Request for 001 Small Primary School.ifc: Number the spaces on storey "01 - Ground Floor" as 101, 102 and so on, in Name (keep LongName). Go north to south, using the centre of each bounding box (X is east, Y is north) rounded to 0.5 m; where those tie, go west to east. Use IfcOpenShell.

First a look at what the model holds.

```python
import ifcopenshell
import ifcopenshell.util.element
import ifcopenshell.util.placement

model = ifcopenshell.open("001 Small Primary School.ifc")
print(model.schema)
storey = next(s for s in model.by_type("IfcBuildingStorey") if s.Name == "01 - Ground Floor")
spaces = [e for e in ifcopenshell.util.element.get_decomposition(storey) if e.is_a("IfcSpace")]
for e in sorted(spaces, key=lambda e: e.id()):
    origin = ifcopenshell.util.placement.get_local_placement(e.ObjectPlacement)[:3, 3]
    print(e.id(), e.Name, e.LongName, origin.round(2) + 0.0, sep=" | ")
```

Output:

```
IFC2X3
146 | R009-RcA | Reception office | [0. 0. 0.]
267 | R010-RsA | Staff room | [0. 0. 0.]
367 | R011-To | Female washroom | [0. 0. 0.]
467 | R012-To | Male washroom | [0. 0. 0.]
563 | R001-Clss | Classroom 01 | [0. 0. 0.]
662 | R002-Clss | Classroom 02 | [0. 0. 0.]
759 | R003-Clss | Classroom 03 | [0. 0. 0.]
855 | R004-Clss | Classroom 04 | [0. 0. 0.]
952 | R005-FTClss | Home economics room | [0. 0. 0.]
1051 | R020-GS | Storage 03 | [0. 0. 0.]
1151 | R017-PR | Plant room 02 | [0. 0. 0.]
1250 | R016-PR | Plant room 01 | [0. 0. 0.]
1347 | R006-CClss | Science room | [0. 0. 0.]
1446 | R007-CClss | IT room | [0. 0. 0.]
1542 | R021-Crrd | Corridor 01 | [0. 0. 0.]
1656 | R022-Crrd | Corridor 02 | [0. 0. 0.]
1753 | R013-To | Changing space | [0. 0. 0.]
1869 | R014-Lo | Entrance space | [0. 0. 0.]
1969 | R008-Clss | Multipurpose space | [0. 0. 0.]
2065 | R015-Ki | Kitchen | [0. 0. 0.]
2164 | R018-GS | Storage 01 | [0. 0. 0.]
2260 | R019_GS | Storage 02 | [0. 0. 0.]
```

```python
import ifcopenshell
import ifcopenshell.geom
import ifcopenshell.util.element
import ifcopenshell.util.shape

model = ifcopenshell.open("001 Small Primary School.ifc")
settings = ifcopenshell.geom.settings()
settings.set("use-world-coords", True)


def centre(element):
    shape = ifcopenshell.geom.create_shape(settings, element)
    return ifcopenshell.util.shape.get_bbox_centroid(shape.geometry)


storey = next(s for s in model.by_type("IfcBuildingStorey") if s.Name == "01 - Ground Floor")
spaces = [e for e in ifcopenshell.util.element.get_decomposition(storey) if e.is_a("IfcSpace")]

# Insertion points can sit at a corner or the storey origin, so sort by the geometry (in metres).
centres = {e: centre(e) for e in spaces}
spaces.sort(key=lambda e: (-round(centres[e][1] / 0.5), centres[e][0]))

for i, e in enumerate(spaces, start=1):
    number = f"1{i:02d}"
    e.Name = number
    print(e.id(), number)

model.write("001 Small Primary School_edited.ifc")
```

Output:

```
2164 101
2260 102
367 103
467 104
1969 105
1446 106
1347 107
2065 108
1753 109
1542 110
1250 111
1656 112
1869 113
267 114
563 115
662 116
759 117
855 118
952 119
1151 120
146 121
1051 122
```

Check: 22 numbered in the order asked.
